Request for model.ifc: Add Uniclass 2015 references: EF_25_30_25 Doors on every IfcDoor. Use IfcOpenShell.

First a look at what the model holds.

```python
import ifcopenshell

model = ifcopenshell.open("model.ifc")
print(model.schema)
print("classifications:", [c.Name for c in model.by_type("IfcClassification")])
for ifc_class in ("IfcDoor", "IfcRoof", "IfcStair", "IfcWall", "IfcWindow"):
    print(ifc_class, len(model.by_type(ifc_class)))
```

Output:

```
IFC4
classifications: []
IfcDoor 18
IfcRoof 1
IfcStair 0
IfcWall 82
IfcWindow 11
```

```python
import ifcopenshell
import ifcopenshell.api.classification

model = ifcopenshell.open("model.ifc")

system = ifcopenshell.api.classification.add_classification(model, classification="Uniclass 2015")

codes = {
    "IfcDoor": ("EF_25_30_25", "Doors"),
}
for ifc_class, (code, name) in codes.items():
    products = model.by_type(ifc_class)
    ifcopenshell.api.classification.add_reference(
        model, products=products, classification=system, identification=code, name=name
    )
    print(code, len(products))

model.write("model-out.ifc")
```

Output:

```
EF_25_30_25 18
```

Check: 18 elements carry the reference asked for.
